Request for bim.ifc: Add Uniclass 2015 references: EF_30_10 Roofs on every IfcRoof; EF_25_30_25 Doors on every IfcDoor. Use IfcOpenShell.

First a look at what the model holds.

```python
import ifcopenshell

model = ifcopenshell.open("bim.ifc")
print(model.schema)
print("classifications:", [c.Name for c in model.by_type("IfcClassification")])
for ifc_class in ("IfcDoor", "IfcRoof", "IfcStair", "IfcWall", "IfcWindow"):
    print(ifc_class, len(model.by_type(ifc_class)))
```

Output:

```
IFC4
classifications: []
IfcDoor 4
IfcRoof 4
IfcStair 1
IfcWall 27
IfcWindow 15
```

```python
import ifcopenshell
import ifcopenshell.api.classification

model = ifcopenshell.open("bim.ifc")

system = ifcopenshell.api.classification.add_classification(model, classification="Uniclass 2015")

codes = {
    "IfcRoof": ("EF_30_10", "Roofs"),
    "IfcDoor": ("EF_25_30_25", "Doors"),
}
for ifc_class, (code, name) in codes.items():
    products = model.by_type(ifc_class)
    ifcopenshell.api.classification.add_reference(
        model, products=products, classification=system, identification=code, name=name
    )
    print(code, len(products))

model.write("bim_edited.ifc")
```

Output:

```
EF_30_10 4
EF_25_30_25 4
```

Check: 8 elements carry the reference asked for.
